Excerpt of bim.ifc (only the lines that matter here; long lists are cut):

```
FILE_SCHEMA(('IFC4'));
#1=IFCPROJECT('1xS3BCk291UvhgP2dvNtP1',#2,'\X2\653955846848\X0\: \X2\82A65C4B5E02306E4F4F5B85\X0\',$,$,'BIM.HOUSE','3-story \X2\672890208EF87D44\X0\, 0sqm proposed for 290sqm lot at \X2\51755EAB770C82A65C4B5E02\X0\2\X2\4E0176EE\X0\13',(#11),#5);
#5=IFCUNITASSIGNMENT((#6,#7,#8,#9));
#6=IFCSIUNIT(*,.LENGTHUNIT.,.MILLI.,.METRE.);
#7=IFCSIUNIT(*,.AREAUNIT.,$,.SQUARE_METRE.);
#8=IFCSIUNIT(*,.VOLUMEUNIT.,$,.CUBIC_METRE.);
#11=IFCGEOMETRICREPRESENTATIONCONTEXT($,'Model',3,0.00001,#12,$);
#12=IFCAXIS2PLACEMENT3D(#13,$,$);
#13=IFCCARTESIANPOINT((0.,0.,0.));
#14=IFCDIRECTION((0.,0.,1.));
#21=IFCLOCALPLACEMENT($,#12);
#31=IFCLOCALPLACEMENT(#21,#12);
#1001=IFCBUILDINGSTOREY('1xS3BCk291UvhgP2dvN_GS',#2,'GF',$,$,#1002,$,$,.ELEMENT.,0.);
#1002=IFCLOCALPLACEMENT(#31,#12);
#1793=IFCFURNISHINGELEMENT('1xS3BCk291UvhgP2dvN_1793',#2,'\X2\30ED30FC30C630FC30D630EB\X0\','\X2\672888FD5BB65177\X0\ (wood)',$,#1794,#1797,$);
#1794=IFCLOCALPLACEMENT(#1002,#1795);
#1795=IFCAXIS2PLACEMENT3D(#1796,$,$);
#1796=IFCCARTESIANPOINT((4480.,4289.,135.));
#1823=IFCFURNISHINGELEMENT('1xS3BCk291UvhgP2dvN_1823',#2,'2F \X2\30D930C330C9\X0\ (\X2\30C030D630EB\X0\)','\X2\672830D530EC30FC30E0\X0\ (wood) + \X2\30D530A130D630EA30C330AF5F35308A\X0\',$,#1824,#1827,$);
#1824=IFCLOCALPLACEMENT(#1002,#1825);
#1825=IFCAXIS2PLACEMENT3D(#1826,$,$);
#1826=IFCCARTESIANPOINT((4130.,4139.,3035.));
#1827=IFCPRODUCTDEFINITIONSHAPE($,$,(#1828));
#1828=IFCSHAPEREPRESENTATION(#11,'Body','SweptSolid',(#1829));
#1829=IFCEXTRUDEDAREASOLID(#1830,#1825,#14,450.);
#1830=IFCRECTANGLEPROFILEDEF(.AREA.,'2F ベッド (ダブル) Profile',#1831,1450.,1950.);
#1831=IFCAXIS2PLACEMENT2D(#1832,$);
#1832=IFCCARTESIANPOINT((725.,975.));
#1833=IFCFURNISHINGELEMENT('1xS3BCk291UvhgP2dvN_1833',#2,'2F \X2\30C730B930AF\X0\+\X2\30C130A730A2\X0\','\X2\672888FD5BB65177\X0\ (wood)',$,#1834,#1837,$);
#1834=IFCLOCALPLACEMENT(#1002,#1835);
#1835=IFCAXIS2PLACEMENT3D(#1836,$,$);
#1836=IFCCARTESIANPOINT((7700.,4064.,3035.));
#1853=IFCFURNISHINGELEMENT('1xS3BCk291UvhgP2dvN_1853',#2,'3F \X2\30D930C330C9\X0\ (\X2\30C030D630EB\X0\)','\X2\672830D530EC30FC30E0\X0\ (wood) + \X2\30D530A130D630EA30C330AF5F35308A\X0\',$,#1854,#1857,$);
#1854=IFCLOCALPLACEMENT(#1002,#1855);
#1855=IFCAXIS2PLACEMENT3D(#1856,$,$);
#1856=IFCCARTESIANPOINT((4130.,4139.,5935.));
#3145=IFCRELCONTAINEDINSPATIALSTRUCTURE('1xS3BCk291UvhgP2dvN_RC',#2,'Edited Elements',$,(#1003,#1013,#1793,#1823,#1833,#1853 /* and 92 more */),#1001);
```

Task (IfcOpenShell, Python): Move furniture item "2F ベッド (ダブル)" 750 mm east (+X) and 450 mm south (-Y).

```python
import ifcopenshell
import ifcopenshell.api.geometry
import ifcopenshell.util.placement
import ifcopenshell.util.unit

model = ifcopenshell.open("bim.ifc")
unit_scale = ifcopenshell.util.unit.calculate_unit_scale(model)

item = model.by_guid("1xS3BCk291UvhgP2dvN_1823")
matrix = ifcopenshell.util.placement.get_local_placement(item.ObjectPlacement)
matrix[0, 3] += 0.75 / unit_scale
matrix[1, 3] -= 0.45 / unit_scale
ifcopenshell.api.geometry.edit_object_placement(model, product=item, matrix=matrix, is_si=False)

print(ifcopenshell.util.placement.get_local_placement(item.ObjectPlacement).round(3) + 0.0)

model.write("bim_updated.ifc")
```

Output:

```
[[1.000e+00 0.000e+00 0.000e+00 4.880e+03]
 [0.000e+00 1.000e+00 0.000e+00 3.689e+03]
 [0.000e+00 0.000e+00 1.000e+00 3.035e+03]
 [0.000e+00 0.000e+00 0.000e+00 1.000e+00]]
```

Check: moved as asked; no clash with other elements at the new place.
